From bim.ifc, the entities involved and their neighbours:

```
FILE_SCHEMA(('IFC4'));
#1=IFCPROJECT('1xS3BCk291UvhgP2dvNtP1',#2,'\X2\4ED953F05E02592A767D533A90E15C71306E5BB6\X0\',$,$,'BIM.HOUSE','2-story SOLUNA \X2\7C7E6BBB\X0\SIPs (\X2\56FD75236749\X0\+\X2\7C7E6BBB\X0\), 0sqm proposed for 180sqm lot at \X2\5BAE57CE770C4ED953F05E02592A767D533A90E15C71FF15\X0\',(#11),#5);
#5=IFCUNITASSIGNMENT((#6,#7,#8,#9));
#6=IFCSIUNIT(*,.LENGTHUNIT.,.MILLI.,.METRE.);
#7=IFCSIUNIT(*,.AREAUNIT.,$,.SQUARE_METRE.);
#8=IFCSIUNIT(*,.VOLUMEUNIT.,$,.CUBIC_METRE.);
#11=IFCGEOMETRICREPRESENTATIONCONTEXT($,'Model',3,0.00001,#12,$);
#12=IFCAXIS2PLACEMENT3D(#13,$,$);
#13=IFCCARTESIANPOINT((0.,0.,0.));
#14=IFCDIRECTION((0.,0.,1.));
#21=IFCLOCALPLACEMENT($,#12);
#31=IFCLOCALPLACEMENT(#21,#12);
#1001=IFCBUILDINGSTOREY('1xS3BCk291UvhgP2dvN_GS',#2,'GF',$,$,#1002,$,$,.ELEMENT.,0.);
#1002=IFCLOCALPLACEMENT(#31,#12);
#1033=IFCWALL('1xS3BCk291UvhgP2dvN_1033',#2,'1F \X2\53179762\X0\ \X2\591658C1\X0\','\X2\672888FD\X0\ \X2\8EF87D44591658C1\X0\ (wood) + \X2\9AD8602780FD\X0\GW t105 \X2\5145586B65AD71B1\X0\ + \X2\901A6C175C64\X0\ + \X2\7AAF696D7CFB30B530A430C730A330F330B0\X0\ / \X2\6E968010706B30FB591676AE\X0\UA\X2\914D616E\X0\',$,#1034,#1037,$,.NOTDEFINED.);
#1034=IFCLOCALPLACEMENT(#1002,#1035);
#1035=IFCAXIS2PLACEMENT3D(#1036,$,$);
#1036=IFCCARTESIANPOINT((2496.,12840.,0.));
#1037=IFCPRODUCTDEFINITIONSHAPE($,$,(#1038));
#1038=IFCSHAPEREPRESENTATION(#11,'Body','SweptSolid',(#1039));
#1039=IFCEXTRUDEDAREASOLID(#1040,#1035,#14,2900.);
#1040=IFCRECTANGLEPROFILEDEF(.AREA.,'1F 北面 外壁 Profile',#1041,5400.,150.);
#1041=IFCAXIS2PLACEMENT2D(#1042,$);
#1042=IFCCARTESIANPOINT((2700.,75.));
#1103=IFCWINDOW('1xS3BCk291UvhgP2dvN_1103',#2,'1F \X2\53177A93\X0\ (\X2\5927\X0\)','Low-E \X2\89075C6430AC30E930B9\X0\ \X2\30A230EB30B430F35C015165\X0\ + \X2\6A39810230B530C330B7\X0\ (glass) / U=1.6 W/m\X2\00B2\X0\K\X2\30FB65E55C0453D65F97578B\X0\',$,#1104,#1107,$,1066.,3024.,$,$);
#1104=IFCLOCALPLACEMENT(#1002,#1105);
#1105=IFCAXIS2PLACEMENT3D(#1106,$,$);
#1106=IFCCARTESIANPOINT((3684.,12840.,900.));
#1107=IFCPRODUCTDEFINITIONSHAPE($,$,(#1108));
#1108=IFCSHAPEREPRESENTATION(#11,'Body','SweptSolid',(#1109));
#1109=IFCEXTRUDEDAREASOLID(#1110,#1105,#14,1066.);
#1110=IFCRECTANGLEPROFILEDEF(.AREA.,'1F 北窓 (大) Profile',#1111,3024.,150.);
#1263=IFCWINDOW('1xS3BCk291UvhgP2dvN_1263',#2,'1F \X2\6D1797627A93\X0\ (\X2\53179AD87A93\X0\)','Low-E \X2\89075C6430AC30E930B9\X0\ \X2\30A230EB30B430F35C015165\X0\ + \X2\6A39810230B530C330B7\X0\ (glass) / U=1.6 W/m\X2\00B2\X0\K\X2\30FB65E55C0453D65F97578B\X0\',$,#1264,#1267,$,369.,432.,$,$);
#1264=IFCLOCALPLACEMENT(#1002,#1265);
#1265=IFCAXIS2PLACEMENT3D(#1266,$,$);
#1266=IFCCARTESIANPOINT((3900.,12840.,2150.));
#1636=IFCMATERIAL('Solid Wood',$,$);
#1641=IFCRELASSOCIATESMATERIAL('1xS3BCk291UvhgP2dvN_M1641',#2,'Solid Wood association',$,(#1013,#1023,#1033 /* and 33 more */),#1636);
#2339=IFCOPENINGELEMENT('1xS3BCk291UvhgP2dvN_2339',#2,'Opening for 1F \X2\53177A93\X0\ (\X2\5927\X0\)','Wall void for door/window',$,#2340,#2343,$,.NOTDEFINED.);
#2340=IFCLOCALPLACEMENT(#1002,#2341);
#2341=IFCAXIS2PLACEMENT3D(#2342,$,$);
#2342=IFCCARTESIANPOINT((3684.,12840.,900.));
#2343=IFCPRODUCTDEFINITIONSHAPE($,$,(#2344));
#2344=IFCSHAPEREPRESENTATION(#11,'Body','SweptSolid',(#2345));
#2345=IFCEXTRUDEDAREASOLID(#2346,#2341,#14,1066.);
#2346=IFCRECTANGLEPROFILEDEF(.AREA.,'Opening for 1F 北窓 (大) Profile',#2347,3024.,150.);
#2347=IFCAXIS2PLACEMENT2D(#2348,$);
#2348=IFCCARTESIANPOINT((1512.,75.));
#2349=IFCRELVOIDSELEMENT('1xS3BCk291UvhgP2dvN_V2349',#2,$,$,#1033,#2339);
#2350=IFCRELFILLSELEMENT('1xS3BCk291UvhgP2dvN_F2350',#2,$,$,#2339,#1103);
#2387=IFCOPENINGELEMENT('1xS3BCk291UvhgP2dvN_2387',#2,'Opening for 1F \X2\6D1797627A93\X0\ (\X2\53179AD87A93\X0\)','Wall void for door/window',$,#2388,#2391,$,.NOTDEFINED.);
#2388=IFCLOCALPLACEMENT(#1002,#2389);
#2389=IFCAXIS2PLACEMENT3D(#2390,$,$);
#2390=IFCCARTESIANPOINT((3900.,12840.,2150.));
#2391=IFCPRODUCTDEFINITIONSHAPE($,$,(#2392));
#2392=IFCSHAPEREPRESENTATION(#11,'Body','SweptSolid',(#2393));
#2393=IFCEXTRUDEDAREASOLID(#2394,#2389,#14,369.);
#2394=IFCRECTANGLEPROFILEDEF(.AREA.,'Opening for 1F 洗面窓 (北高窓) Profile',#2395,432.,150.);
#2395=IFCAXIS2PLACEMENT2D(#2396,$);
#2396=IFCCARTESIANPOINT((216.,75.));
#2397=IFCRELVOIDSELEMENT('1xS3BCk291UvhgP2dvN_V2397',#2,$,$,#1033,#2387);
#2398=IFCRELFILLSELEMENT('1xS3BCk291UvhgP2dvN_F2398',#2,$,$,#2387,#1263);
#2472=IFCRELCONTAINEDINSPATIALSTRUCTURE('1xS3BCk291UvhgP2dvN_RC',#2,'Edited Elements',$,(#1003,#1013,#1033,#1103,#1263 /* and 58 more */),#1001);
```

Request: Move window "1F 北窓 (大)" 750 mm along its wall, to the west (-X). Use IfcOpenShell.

```python
import ifcopenshell
import ifcopenshell.api.geometry
import ifcopenshell.util.placement
import ifcopenshell.util.unit

model = ifcopenshell.open("bim.ifc")
unit_scale = ifcopenshell.util.unit.calculate_unit_scale(model)

window = model.by_guid("1xS3BCk291UvhgP2dvN_1103")
opening = window.FillsVoids[0].RelatingOpeningElement
wall = opening.VoidsElements[0].RelatingBuildingElement

wall_matrix = ifcopenshell.util.placement.get_local_placement(wall.ObjectPlacement)
shift = wall_matrix[:3, 0] * -0.75 / unit_scale
before = ifcopenshell.util.placement.get_local_placement(window.ObjectPlacement)[:3, 3].copy()

# The window is not placed relative to its opening, so move both.
for product in (opening, window):
    matrix = ifcopenshell.util.placement.get_local_placement(product.ObjectPlacement)
    matrix[:3, 3] += shift
    ifcopenshell.api.geometry.edit_object_placement(model, product=product, matrix=matrix, is_si=False)

after = ifcopenshell.util.placement.get_local_placement(window.ObjectPlacement)[:3, 3]
print("window moved by", (after - before).round(3) + 0.0)

model.write("bim_v2.ifc")
```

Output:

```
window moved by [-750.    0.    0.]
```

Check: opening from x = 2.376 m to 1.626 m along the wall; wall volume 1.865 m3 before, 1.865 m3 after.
